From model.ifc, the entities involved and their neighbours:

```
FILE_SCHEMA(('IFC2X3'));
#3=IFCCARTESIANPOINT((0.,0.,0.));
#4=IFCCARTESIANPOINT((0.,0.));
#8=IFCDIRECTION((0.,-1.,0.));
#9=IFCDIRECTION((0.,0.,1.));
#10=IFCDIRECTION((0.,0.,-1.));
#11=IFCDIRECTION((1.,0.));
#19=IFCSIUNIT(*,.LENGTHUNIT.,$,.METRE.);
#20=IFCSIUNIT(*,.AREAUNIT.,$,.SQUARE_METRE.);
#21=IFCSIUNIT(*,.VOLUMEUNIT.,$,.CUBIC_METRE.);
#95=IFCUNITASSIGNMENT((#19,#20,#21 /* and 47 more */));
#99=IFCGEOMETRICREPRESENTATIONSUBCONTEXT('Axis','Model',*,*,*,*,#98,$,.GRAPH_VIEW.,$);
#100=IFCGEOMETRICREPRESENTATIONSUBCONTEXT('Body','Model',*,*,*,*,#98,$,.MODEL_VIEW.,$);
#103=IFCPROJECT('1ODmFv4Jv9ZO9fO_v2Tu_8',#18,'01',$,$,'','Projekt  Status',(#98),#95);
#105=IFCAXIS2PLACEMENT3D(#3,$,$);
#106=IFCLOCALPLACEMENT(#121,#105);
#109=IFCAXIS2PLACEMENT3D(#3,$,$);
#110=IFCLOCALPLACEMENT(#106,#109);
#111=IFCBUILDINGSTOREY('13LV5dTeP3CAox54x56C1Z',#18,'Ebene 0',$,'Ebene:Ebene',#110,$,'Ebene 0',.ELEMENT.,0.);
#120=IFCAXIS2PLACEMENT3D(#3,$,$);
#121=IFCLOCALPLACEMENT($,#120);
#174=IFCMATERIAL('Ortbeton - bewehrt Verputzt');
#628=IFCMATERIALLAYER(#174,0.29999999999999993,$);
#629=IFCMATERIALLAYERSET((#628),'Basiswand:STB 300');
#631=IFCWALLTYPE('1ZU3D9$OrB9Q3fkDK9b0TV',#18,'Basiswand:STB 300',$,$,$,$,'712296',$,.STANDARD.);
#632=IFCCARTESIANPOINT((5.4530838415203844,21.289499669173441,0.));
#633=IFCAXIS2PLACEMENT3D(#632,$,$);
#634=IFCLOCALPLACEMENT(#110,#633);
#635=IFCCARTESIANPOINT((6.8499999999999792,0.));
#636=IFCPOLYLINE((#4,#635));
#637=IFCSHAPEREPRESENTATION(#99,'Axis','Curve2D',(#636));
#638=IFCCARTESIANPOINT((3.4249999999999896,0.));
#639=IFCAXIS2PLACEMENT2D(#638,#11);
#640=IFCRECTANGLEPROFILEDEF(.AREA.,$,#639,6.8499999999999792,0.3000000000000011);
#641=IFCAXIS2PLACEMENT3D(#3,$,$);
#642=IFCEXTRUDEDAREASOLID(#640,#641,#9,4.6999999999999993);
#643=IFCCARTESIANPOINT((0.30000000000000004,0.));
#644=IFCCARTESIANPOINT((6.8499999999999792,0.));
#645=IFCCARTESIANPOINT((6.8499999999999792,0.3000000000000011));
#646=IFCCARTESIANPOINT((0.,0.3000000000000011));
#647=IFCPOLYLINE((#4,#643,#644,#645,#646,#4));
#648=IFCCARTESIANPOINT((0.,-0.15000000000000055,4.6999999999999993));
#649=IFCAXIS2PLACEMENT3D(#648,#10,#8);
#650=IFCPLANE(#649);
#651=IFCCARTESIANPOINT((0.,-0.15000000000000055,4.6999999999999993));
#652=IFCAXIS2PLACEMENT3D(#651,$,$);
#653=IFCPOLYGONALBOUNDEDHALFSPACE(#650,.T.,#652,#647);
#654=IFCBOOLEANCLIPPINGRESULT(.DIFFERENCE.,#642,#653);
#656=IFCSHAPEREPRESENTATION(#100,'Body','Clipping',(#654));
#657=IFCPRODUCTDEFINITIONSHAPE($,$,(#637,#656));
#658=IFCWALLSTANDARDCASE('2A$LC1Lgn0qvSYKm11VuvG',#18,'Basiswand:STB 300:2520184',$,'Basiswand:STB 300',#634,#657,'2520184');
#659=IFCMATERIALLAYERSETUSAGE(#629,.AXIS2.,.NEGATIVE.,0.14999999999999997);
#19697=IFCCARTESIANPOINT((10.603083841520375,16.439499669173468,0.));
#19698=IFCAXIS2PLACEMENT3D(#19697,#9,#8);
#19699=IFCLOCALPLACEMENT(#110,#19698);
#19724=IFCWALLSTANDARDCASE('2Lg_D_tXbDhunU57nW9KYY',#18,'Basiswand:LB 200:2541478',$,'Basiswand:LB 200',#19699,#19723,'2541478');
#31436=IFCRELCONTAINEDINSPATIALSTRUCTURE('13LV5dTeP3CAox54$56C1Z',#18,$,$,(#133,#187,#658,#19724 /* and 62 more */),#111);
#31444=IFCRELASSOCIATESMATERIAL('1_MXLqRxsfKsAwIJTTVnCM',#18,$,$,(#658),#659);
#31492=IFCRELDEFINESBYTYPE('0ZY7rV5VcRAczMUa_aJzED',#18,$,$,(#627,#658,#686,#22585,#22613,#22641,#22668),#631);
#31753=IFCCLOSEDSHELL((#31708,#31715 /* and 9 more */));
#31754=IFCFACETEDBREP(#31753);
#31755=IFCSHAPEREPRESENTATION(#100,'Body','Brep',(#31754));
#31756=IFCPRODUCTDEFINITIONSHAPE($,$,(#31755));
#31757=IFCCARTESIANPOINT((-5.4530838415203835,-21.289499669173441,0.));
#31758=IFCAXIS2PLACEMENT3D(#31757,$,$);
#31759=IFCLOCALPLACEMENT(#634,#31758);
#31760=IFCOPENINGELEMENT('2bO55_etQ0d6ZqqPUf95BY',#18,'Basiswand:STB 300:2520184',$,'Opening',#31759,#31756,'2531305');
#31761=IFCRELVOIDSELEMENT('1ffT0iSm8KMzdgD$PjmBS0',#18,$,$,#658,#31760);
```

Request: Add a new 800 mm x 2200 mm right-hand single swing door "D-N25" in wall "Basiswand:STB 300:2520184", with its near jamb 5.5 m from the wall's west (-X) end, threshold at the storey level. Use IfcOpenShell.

```python
import numpy as np
import ifcopenshell
import ifcopenshell.api.feature
import ifcopenshell.api.geometry
import ifcopenshell.api.root
import ifcopenshell.api.spatial
import ifcopenshell.api.type
import ifcopenshell.geom
import ifcopenshell.util.element
import ifcopenshell.util.placement
import ifcopenshell.util.representation
import ifcopenshell.util.shape
import ifcopenshell.util.unit

model = ifcopenshell.open("model.ifc")
unit_scale = ifcopenshell.util.unit.calculate_unit_scale(model)
settings = ifcopenshell.geom.settings()


def volume(element):
    """Net volume in cubic metres, openings subtracted."""
    shape = ifcopenshell.geom.create_shape(settings, element)
    return ifcopenshell.util.shape.get_volume(shape.geometry)


wall = model.by_id(658)
storey = ifcopenshell.util.element.get_container(wall, ifc_class="IfcBuildingStorey")
context = ifcopenshell.util.representation.get_context(model, "Model", "Body", "MODEL_VIEW")
before = volume(wall)

width, height, from_end, sill = 0.8, 2.2, 5.5, 0.0  # metres

# The wall runs along its own X axis, and the end named is its -X end.
wall_shape = ifcopenshell.geom.create_shape(settings, wall)
x, y, z = ifcopenshell.util.shape.get_vertices(wall_shape.geometry).T
start = x.min() + from_end
face, thickness = float(y.min()), float(y.max() - y.min())
wall_matrix = ifcopenshell.util.placement.get_local_placement(wall.ObjectPlacement)
level = ifcopenshell.util.placement.get_local_placement(storey.ObjectPlacement)[2, 3]


def in_wall(x, y):
    """Placement at x, y metres in the wall's axes, at sill height."""
    matrix = wall_matrix.copy()
    matrix[:, 3] = wall_matrix @ np.array([x / unit_scale, y / unit_scale, 0.0, 1.0])
    matrix[2, 3] = level + sill / unit_scale
    return matrix


# Opening: a box that overshoots both wall faces by 50 mm.
opening = ifcopenshell.api.root.create_entity(model, ifc_class="IfcOpeningElement")
box = ifcopenshell.api.geometry.add_wall_representation(
    model, context=context, length=width, height=height, thickness=thickness + 0.1
)
ifcopenshell.api.geometry.assign_representation(model, product=opening, representation=box)
ifcopenshell.api.geometry.edit_object_placement(model, product=opening, matrix=in_wall(start, face - 0.05), is_si=False)
ifcopenshell.api.feature.add_feature(model, feature=opening, element=wall)

door = ifcopenshell.api.root.create_entity(model, ifc_class="IfcDoor", name="D-N25")
door.OverallWidth, door.OverallHeight = width / unit_scale, height / unit_scale
body = ifcopenshell.api.geometry.add_door_representation(
    model,
    context=context,
    overall_width=door.OverallWidth,
    overall_height=door.OverallHeight,
    operation_type="SINGLE_SWING_RIGHT",
    lining_properties={"LiningDepth": thickness / unit_scale, "ThresholdDepth": thickness / unit_scale},
)
ifcopenshell.api.geometry.assign_representation(model, product=door, representation=body)
ifcopenshell.api.spatial.assign_container(model, products=[door], relating_structure=storey)
fills = ifcopenshell.api.feature.add_filling(model, opening=opening, element=door)
fills.OwnerHistory = door.OwnerHistory  # required in IFC2X3

# IFC2X3 keeps the operation on the door style.
style = ifcopenshell.api.root.create_entity(model, ifc_class="IfcDoorStyle", name="D-N25")
style.OperationType, style.ConstructionType = "SINGLE_SWING_RIGHT", "NOTDEFINED"
style.ParameterTakesPrecedence = style.Sizeable = False
ifcopenshell.api.type.assign_type(model, related_objects=[door], relating_type=style)

# The lining spans the wall, so the door starts at the wall face.
ifcopenshell.api.geometry.edit_object_placement(model, product=door, matrix=in_wall(start, face), is_si=False)

after = volume(wall)

print(f"wall volume {before:.3f} -> {after:.3f} m3")

model.write("model_edited.ifc")
```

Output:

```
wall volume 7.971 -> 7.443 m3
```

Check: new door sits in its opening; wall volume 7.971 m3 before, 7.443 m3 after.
